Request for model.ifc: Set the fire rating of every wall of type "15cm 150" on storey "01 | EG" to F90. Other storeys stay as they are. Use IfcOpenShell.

First a look at what the model holds.

```python
import ifcopenshell
import ifcopenshell.util.element

model = ifcopenshell.open("model.ifc")
print(model.schema)
storey = next(s for s in model.by_type("IfcBuildingStorey") if s.Name == "01 | EG")
walls = [e for e in ifcopenshell.util.element.get_decomposition(storey) if e.is_a("IfcWall")]
seen = {}
for e in walls:
    element_type = ifcopenshell.util.element.get_type(e)
    key = (element_type.Name if element_type != e and element_type else None, ifcopenshell.util.element.get_pset(e, "Pset_WallCommon", "FireRating"))
    seen[key] = seen.get(key, 0) + 1
for (name, value), count in sorted(seen.items(), key=str):
    print(count, "x", name, "|", value)
```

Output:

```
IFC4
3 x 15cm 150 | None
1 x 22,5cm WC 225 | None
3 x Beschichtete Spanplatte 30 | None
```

```python
import ifcopenshell
import ifcopenshell.api.pset
import ifcopenshell.util.element

model = ifcopenshell.open("model.ifc")

storey = next(s for s in model.by_type("IfcBuildingStorey") if s.Name == "01 | EG")
walls = [e for e in ifcopenshell.util.element.get_decomposition(storey) if e.is_a("IfcWall")]

count = 0
for e in walls:
    element_type = ifcopenshell.util.element.get_type(e)
    if element_type in (None, e) or element_type.Name != "15cm 150":
        continue
    # add_pset returns the element's existing set when there is one.
    pset = ifcopenshell.api.pset.add_pset(model, product=e, name="Pset_WallCommon")
    ifcopenshell.api.pset.edit_pset(model, pset=pset, properties={"FireRating": "F90"})
    count += 1

print(count, "walls updated")

model.write("model_rev.ifc")
```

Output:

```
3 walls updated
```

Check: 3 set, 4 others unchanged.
